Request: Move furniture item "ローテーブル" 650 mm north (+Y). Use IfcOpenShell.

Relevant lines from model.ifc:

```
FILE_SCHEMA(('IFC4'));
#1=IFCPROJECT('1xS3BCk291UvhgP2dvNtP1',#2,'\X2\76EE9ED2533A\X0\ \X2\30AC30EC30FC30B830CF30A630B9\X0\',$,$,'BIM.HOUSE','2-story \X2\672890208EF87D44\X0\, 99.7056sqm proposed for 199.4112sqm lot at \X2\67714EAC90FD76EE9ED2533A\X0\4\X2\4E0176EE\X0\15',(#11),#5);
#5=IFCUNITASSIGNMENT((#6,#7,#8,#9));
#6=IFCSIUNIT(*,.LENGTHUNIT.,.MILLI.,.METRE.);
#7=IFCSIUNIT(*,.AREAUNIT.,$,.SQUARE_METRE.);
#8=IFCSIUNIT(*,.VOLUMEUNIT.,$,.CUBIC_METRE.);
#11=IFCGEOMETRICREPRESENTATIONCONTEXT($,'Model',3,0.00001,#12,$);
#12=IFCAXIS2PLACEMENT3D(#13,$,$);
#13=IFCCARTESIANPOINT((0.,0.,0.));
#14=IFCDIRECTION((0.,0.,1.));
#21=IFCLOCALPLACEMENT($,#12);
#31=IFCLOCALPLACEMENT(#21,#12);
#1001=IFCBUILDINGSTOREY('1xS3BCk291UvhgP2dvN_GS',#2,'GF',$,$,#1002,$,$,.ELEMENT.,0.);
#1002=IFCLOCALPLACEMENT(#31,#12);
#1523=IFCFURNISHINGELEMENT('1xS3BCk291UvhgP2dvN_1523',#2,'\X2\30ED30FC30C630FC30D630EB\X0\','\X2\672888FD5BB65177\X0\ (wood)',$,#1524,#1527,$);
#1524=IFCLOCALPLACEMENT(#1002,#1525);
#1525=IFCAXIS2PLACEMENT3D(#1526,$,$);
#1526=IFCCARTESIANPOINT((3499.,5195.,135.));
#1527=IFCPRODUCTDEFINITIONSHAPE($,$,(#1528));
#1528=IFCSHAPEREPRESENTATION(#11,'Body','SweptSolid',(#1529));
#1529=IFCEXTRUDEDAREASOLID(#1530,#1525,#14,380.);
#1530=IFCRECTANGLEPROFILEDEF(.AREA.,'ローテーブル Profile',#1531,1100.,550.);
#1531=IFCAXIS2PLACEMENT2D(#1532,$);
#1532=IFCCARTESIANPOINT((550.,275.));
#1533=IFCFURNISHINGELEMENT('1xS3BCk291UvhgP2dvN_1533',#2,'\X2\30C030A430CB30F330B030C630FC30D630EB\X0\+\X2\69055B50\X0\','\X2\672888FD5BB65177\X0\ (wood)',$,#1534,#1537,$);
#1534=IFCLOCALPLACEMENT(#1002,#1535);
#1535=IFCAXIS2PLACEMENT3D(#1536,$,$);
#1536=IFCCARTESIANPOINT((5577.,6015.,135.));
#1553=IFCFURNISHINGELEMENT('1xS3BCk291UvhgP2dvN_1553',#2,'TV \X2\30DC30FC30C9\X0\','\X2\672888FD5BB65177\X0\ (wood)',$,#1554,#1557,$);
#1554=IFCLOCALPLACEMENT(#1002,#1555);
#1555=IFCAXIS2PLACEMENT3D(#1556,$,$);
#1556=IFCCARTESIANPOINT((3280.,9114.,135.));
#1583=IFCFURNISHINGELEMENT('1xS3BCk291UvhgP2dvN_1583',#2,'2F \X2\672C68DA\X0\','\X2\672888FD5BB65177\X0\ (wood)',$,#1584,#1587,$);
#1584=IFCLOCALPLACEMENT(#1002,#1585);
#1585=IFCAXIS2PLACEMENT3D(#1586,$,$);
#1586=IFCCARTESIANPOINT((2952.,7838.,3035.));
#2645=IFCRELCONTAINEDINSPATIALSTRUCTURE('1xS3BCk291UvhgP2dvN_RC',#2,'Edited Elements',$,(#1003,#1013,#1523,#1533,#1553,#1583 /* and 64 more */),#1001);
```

```python
import ifcopenshell
import ifcopenshell.api.geometry
import ifcopenshell.util.placement
import ifcopenshell.util.unit

model = ifcopenshell.open("model.ifc")
unit_scale = ifcopenshell.util.unit.calculate_unit_scale(model)

item = model.by_guid("1xS3BCk291UvhgP2dvN_1523")
matrix = ifcopenshell.util.placement.get_local_placement(item.ObjectPlacement)
matrix[1, 3] += 0.65 / unit_scale
ifcopenshell.api.geometry.edit_object_placement(model, product=item, matrix=matrix, is_si=False)

print(ifcopenshell.util.placement.get_local_placement(item.ObjectPlacement).round(3) + 0.0)

model.write("model-out.ifc")
```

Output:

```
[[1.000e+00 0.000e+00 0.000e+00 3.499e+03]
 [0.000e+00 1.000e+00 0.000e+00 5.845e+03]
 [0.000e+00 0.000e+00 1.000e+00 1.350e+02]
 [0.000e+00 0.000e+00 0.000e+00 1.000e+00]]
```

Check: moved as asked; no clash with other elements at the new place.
